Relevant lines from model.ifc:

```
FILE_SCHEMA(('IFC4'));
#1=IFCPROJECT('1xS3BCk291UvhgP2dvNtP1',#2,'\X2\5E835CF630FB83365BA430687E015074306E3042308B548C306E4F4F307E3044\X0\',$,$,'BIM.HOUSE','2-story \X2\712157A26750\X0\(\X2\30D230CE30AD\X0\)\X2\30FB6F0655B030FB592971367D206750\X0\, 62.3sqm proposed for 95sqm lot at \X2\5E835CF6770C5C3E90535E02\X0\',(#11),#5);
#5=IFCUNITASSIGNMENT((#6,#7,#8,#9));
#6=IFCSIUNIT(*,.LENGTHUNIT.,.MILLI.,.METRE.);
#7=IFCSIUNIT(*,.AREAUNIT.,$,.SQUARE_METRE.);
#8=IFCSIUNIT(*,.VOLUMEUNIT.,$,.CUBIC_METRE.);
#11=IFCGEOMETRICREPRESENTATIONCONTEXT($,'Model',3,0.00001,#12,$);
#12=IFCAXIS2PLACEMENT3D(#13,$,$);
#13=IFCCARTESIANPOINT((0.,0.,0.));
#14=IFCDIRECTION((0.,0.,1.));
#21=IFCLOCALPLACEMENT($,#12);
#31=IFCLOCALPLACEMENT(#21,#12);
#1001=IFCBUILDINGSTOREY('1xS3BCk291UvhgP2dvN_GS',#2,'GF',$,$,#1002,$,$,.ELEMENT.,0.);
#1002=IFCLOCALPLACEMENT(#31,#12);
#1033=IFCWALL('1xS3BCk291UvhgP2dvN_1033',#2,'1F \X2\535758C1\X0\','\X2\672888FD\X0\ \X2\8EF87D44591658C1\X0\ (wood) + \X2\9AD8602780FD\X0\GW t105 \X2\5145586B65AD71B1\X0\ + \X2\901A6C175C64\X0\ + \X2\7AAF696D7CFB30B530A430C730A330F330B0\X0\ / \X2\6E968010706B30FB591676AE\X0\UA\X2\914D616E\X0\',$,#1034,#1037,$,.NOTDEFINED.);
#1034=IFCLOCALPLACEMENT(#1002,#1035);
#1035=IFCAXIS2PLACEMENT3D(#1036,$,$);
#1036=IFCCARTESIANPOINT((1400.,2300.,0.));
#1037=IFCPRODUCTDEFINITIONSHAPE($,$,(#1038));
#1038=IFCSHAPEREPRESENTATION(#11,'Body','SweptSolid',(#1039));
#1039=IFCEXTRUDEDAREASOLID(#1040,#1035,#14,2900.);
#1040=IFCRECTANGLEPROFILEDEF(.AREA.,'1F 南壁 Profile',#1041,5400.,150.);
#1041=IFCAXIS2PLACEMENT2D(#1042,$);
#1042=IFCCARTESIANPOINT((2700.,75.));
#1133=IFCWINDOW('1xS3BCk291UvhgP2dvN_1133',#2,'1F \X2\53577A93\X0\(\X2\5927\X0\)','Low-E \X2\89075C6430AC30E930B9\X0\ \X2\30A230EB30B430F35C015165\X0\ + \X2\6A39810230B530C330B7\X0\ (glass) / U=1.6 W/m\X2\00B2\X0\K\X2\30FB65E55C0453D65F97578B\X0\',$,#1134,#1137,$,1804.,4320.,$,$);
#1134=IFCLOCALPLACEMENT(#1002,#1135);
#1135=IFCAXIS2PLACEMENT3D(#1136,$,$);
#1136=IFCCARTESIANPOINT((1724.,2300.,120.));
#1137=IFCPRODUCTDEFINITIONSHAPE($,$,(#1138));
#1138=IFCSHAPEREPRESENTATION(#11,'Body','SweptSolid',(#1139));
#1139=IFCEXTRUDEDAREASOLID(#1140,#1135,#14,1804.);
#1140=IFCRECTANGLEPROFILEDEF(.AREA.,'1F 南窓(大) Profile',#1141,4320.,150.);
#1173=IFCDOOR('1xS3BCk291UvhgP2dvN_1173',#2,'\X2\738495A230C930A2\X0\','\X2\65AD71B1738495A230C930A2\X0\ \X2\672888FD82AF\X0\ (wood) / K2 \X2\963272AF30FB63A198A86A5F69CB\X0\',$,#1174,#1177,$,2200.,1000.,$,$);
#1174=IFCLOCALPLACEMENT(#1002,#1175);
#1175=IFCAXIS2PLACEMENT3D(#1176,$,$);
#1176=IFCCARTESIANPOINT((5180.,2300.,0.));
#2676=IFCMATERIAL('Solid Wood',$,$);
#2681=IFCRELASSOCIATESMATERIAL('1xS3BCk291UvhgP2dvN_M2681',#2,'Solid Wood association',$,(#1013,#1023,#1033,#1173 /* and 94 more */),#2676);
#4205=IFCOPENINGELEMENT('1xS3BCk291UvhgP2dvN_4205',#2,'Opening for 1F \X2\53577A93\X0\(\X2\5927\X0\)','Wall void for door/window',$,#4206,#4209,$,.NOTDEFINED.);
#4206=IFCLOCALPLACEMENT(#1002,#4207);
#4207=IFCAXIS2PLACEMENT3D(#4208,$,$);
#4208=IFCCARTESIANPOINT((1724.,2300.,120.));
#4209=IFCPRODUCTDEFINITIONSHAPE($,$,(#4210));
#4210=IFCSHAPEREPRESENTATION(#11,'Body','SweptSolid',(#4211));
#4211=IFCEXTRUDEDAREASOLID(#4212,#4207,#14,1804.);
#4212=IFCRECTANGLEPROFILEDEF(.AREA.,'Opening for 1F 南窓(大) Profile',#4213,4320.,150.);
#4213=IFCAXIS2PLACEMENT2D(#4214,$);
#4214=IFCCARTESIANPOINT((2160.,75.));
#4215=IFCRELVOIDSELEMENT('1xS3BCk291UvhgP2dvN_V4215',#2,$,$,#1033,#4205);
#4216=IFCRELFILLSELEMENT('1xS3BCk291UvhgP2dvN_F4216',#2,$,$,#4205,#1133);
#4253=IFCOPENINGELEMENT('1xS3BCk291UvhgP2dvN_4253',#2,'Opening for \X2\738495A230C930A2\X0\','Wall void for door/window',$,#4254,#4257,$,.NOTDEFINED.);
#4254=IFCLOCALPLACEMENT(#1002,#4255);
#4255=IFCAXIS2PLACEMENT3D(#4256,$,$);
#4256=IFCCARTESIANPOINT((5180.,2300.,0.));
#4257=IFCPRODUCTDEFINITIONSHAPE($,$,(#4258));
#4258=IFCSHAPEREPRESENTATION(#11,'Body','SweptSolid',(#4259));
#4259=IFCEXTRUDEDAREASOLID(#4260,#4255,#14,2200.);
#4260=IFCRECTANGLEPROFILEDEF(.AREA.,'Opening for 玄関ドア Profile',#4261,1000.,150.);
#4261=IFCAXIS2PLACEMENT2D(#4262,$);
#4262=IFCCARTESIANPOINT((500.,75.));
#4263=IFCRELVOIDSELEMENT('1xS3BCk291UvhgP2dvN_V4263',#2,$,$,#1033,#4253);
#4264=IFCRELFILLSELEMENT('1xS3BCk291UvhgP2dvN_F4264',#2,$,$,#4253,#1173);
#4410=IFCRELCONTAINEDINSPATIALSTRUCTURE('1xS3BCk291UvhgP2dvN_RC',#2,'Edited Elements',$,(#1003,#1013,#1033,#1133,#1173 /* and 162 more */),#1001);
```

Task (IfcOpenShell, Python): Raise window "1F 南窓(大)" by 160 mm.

```python
import numpy as np
import ifcopenshell
import ifcopenshell.api.geometry
import ifcopenshell.util.placement
import ifcopenshell.util.unit

model = ifcopenshell.open("model.ifc")
unit_scale = ifcopenshell.util.unit.calculate_unit_scale(model)

window = model.by_guid("1xS3BCk291UvhgP2dvN_1133")
opening = window.FillsVoids[0].RelatingOpeningElement
dz = 160.0

shift = np.array([0.0, 0.0, dz])
# The window is not placed relative to its opening, so move both.
for product in (opening, window):
    matrix = ifcopenshell.util.placement.get_local_placement(product.ObjectPlacement)
    matrix[:3, 3] += shift
    ifcopenshell.api.geometry.edit_object_placement(model, product=product, matrix=matrix, is_si=False)

print(f"moved by {dz * unit_scale:+.3f} m")

model.write("model_edited.ifc")
```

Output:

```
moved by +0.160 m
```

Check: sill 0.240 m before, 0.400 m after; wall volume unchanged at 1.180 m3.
